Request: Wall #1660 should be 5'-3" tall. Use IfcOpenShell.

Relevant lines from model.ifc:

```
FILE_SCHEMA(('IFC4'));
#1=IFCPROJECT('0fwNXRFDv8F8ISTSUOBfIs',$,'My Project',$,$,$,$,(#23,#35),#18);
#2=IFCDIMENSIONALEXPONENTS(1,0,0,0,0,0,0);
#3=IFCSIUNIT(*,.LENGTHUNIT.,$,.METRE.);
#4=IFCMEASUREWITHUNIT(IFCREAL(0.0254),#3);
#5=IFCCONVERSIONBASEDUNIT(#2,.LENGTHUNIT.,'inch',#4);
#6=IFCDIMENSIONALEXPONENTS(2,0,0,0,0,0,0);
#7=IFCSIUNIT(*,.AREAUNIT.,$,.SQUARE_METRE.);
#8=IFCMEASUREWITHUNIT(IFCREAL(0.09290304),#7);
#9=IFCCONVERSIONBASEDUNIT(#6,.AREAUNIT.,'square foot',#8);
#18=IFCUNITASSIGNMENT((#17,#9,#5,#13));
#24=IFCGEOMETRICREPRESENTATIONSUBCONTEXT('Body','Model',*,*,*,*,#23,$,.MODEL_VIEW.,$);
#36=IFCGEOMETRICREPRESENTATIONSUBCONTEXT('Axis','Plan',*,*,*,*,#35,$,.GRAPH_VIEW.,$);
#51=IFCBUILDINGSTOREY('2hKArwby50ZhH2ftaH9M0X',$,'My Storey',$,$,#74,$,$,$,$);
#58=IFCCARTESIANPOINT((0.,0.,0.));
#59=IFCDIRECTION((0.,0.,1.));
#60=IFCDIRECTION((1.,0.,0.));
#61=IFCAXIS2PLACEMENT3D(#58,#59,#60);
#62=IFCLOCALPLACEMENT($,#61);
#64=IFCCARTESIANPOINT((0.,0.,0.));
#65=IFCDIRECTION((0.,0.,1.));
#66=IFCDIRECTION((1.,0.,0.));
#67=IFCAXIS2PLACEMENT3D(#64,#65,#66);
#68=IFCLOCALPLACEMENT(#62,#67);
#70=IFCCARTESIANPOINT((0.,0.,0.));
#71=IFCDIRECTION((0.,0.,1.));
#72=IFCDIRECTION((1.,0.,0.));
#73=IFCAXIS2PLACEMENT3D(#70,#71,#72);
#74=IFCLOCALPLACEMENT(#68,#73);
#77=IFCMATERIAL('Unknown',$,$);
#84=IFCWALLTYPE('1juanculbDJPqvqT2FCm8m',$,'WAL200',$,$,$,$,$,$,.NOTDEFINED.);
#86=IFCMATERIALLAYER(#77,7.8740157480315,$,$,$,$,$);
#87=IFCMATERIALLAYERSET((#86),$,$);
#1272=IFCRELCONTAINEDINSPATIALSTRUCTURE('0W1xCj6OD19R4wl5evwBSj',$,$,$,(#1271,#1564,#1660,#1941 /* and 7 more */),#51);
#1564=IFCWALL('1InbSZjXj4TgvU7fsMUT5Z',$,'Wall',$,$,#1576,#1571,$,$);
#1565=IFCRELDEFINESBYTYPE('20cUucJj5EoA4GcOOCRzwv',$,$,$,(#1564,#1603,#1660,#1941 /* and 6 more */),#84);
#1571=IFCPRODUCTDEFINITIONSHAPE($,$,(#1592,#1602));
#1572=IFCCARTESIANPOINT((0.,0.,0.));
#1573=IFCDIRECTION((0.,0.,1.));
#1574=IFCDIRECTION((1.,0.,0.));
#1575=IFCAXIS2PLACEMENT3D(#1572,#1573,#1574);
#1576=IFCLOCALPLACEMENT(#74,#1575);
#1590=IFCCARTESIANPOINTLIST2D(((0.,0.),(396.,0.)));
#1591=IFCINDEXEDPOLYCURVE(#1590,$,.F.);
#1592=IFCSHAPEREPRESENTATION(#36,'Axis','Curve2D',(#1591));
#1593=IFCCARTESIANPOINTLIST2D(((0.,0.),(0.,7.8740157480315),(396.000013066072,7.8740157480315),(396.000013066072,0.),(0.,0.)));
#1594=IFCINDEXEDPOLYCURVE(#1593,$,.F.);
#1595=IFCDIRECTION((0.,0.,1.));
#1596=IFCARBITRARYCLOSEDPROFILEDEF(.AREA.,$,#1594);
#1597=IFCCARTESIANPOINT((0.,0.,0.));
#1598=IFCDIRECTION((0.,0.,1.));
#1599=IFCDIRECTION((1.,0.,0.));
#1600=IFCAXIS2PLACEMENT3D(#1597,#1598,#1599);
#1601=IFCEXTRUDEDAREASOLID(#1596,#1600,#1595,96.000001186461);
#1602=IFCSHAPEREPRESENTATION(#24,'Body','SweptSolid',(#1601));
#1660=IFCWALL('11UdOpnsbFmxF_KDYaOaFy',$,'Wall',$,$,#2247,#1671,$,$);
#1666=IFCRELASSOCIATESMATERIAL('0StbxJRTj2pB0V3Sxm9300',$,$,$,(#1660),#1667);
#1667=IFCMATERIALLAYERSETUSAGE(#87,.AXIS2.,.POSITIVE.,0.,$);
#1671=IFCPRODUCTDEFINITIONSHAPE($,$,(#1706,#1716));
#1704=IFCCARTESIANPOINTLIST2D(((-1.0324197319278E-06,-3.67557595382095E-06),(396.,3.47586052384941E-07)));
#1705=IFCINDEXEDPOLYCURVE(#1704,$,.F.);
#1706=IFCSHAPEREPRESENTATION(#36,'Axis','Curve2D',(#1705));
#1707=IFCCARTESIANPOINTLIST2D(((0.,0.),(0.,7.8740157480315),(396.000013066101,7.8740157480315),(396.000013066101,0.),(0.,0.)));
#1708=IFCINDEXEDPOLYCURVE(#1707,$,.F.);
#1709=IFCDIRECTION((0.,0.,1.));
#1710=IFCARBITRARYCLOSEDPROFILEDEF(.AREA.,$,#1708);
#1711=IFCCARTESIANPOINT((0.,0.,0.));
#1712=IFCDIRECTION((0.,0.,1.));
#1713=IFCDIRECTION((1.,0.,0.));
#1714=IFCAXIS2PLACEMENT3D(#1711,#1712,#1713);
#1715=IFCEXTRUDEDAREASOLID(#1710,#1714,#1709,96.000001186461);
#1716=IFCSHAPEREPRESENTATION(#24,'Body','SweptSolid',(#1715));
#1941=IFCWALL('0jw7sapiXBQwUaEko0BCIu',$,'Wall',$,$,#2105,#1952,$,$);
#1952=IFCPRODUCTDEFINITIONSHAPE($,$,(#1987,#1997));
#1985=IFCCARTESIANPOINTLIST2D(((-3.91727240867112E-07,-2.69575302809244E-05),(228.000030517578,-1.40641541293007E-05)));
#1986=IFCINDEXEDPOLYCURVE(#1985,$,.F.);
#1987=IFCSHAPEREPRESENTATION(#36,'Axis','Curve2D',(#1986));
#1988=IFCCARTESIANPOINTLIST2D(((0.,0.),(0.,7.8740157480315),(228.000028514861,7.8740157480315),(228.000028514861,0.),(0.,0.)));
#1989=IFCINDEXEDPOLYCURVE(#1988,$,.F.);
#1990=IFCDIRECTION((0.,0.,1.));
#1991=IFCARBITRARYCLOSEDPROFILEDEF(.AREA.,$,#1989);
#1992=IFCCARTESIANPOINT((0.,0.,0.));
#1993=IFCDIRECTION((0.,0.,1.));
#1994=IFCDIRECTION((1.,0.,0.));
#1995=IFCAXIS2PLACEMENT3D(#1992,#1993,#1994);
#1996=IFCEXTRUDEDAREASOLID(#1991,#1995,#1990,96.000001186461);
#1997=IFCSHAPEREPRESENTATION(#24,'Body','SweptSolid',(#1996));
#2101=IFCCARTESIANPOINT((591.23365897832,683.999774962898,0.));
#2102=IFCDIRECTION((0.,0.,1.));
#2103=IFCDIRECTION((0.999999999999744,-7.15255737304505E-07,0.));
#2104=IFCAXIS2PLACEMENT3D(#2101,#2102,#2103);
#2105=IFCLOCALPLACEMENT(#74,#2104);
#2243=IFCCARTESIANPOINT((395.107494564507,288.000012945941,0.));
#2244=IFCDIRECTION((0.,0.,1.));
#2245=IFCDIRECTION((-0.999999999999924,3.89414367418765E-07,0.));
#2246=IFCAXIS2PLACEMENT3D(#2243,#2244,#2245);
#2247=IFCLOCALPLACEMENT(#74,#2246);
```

```python
import ifcopenshell
import ifcopenshell.geom
import ifcopenshell.util.representation
import ifcopenshell.util.shape
import ifcopenshell.util.unit

model = ifcopenshell.open("model.ifc")
unit_scale = ifcopenshell.util.unit.calculate_unit_scale(model)
settings = ifcopenshell.geom.settings()


def volume(element):
    """Net volume in cubic metres, openings subtracted."""
    shape = ifcopenshell.geom.create_shape(settings, element)
    return ifcopenshell.util.shape.get_volume(shape.geometry)


wall = model.by_guid("11UdOpnsbFmxF_KDYaOaFy")
before = volume(wall)

body = ifcopenshell.util.representation.get_representation(wall, "Model", "Body")
solid = body.Items[0]
old_height = solid.Depth
solid.Depth = 63 * 0.0254 / unit_scale
after = volume(wall)

print(f"height {old_height:g} -> {solid.Depth:g}, volume {before:.3f} -> {after:.3f} m3")

model.write("model_rev.ifc")
```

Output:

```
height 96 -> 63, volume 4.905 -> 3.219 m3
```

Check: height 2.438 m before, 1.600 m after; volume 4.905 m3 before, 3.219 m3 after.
